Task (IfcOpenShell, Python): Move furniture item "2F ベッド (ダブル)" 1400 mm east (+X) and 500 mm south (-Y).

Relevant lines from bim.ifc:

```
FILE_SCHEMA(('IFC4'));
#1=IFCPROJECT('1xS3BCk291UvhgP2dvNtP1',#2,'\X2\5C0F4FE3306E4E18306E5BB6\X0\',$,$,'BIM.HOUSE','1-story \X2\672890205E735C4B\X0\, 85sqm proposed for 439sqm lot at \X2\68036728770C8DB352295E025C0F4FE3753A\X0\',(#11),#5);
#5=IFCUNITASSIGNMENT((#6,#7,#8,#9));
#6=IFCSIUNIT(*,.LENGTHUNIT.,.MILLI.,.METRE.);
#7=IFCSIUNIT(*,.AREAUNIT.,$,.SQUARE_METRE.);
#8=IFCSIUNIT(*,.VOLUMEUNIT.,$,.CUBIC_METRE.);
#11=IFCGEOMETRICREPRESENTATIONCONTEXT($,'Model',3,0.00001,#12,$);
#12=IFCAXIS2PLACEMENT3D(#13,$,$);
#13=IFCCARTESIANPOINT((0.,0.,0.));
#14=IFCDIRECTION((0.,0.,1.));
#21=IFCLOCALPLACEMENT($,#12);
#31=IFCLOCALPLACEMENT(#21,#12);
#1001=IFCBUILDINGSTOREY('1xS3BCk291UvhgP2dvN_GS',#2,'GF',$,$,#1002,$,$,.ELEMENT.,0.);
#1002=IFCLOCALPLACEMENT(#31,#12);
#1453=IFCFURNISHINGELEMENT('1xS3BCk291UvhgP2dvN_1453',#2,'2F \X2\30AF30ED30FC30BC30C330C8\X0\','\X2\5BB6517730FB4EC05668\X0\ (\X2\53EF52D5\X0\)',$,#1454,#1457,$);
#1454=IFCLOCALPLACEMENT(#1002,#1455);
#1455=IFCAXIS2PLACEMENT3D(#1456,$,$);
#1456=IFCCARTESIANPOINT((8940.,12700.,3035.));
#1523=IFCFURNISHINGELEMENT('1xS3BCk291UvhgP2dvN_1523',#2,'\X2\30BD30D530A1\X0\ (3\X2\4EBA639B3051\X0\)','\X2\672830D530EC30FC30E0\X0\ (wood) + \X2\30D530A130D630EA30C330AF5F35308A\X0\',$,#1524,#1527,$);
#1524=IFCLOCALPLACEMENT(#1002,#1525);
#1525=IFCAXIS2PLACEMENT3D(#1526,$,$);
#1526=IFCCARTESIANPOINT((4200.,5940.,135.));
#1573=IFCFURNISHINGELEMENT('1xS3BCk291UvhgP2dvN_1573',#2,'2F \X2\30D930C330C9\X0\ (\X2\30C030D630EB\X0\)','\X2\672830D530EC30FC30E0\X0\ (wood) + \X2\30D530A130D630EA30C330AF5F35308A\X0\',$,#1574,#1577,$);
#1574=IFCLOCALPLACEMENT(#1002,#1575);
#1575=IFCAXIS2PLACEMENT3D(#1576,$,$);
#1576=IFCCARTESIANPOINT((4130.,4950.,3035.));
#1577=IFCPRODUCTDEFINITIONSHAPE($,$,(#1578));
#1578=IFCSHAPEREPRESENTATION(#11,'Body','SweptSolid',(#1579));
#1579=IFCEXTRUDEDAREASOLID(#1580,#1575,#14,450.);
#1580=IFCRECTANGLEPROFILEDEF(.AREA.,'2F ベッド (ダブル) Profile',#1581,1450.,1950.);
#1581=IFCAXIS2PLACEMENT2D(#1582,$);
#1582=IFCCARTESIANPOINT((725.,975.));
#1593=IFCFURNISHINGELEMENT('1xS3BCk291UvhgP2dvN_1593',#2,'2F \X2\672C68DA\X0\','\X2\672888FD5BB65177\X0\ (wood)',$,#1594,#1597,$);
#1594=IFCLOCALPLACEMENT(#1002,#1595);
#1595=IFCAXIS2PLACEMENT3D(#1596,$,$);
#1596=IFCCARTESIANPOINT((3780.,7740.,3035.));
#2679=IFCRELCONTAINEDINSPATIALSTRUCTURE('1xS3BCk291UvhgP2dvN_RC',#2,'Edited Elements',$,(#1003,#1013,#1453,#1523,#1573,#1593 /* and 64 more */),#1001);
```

```python
import ifcopenshell
import ifcopenshell.api.geometry
import ifcopenshell.util.placement
import ifcopenshell.util.unit

model = ifcopenshell.open("bim.ifc")
unit_scale = ifcopenshell.util.unit.calculate_unit_scale(model)

item = model.by_guid("1xS3BCk291UvhgP2dvN_1573")
matrix = ifcopenshell.util.placement.get_local_placement(item.ObjectPlacement)
matrix[0, 3] += 1.4 / unit_scale
matrix[1, 3] -= 0.5 / unit_scale
ifcopenshell.api.geometry.edit_object_placement(model, product=item, matrix=matrix, is_si=False)

print(ifcopenshell.util.placement.get_local_placement(item.ObjectPlacement).round(3) + 0.0)

model.write("bim_rev.ifc")
```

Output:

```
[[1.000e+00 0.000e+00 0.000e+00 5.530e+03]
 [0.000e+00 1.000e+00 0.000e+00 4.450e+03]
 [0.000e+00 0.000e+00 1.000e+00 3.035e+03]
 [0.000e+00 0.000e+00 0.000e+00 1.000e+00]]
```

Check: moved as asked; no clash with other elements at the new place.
